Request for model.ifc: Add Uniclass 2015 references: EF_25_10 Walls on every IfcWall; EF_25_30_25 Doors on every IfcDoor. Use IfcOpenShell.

First a look at what the model holds.

```python
import ifcopenshell

model = ifcopenshell.open("model.ifc")
print(model.schema)
print("classifications:", [c.Name for c in model.by_type("IfcClassification")])
for ifc_class in ("IfcDoor", "IfcRoof", "IfcStair", "IfcWall", "IfcWindow"):
    print(ifc_class, len(model.by_type(ifc_class)))
```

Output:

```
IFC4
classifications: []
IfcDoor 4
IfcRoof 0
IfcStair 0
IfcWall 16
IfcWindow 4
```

```python
import ifcopenshell
import ifcopenshell.api.classification

model = ifcopenshell.open("model.ifc")

system = ifcopenshell.api.classification.add_classification(model, classification="Uniclass 2015")

codes = {
    "IfcWall": ("EF_25_10", "Walls"),
    "IfcDoor": ("EF_25_30_25", "Doors"),
}
for ifc_class, (code, name) in codes.items():
    products = model.by_type(ifc_class)
    ifcopenshell.api.classification.add_reference(
        model, products=products, classification=system, identification=code, name=name
    )
    print(code, len(products))

model.write("model_v2.ifc")
```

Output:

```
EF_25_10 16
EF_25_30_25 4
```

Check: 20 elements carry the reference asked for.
